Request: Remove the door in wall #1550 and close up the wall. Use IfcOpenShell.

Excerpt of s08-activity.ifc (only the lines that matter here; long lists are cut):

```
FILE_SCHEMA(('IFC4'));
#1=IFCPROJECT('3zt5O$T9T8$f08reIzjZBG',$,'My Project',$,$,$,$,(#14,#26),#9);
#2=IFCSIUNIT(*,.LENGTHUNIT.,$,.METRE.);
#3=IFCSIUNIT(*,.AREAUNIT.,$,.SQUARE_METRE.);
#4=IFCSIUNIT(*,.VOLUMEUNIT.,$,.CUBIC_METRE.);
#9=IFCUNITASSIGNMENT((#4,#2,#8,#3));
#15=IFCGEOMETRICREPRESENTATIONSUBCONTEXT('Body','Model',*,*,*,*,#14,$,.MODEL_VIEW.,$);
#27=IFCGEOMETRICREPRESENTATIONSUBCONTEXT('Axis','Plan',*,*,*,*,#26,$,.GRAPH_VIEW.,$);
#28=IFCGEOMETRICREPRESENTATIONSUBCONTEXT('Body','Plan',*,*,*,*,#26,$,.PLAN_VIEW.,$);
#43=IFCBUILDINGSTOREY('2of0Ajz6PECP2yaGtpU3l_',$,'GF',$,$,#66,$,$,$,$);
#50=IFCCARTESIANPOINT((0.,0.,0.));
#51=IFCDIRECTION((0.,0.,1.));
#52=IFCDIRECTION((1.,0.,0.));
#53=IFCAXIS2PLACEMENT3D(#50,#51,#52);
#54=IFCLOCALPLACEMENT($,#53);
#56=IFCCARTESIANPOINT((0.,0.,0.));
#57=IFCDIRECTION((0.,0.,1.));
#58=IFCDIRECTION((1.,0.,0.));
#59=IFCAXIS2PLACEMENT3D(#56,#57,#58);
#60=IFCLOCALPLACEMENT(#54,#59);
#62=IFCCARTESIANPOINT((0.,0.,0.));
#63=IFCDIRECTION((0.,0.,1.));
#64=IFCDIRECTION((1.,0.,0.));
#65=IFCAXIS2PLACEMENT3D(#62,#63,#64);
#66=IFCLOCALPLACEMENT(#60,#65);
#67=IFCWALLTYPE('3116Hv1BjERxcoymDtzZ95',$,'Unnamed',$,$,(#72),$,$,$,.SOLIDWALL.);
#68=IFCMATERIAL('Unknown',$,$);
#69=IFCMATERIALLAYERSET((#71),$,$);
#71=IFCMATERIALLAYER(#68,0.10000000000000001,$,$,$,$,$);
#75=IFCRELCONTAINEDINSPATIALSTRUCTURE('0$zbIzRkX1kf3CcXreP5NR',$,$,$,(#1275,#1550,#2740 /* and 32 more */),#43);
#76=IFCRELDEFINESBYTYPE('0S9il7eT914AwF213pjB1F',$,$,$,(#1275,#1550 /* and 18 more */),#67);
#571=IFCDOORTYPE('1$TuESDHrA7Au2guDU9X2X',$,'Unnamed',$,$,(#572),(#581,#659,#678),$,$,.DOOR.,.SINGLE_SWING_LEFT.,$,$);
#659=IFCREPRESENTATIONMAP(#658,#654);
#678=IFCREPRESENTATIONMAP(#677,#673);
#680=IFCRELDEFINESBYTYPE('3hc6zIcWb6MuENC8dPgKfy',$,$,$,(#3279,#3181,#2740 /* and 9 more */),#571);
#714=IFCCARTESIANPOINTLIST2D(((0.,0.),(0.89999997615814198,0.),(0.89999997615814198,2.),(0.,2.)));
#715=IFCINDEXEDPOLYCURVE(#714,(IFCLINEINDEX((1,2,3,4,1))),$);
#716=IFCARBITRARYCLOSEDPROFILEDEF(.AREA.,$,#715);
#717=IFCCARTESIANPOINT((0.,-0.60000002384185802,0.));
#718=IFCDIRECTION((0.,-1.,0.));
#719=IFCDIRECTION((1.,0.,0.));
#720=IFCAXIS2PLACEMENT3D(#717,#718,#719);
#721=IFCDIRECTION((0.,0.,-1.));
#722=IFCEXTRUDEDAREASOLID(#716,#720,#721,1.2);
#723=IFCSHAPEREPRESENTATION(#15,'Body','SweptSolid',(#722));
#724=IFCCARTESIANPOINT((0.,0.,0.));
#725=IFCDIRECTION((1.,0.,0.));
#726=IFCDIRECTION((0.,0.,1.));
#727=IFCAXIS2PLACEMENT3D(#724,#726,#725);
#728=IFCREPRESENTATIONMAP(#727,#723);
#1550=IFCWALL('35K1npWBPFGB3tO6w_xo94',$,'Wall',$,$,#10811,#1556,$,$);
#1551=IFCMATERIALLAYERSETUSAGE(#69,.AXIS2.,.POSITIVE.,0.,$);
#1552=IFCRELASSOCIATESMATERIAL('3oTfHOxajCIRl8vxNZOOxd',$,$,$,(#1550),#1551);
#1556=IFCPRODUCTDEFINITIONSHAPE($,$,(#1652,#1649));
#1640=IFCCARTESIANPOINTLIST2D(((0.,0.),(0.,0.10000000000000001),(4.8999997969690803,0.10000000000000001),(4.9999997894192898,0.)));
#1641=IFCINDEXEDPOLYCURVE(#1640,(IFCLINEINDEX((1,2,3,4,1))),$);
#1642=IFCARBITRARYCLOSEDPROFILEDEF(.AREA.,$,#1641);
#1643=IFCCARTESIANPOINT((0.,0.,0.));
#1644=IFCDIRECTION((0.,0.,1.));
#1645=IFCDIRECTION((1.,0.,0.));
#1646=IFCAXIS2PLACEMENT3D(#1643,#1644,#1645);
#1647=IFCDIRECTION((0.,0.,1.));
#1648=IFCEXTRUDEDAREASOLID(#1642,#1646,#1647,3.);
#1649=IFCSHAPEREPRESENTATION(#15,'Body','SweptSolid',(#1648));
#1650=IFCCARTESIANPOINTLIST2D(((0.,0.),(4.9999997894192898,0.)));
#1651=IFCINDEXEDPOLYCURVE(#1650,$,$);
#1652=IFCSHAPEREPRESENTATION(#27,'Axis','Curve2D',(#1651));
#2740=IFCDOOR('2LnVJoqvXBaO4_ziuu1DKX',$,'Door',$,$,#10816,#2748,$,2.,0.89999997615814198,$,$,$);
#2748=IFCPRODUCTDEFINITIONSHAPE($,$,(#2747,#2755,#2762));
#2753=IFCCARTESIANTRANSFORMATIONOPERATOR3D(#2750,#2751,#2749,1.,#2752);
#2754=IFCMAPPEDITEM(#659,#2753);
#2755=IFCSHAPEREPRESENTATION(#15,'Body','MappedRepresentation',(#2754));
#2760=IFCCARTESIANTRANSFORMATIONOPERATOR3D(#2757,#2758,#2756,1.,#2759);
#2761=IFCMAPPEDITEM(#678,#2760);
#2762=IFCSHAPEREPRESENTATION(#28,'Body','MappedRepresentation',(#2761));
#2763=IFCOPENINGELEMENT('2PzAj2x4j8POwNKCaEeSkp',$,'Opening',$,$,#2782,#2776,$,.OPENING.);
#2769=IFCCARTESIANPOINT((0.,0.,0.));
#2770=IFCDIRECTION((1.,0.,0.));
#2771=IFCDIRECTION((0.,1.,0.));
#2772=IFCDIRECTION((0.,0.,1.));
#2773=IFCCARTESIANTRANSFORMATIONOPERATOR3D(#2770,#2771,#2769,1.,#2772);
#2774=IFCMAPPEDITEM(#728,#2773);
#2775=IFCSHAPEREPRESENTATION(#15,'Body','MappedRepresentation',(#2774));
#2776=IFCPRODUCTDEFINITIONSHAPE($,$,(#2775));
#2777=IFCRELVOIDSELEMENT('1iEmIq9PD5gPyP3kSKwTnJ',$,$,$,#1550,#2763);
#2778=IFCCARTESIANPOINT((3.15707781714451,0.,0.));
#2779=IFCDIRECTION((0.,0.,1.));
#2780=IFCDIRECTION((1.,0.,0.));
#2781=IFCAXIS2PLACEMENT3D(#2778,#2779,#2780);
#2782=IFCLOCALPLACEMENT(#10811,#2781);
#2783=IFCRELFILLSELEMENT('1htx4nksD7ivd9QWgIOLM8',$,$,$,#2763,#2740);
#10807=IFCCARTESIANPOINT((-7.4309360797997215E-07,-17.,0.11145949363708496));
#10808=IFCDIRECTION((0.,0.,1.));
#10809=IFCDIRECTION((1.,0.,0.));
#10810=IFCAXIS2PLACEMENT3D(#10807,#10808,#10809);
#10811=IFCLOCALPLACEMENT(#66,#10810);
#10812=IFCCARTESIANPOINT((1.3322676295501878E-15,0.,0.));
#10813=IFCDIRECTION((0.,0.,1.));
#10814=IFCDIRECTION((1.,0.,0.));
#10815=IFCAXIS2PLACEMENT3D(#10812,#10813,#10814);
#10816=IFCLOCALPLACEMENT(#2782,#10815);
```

```python
import ifcopenshell
import ifcopenshell.api.feature
import ifcopenshell.api.root
import ifcopenshell.geom
import ifcopenshell.util.shape

model = ifcopenshell.open("s08-activity.ifc")
settings = ifcopenshell.geom.settings()


def volume(element):
    """Net volume in cubic metres, openings subtracted."""
    shape = ifcopenshell.geom.create_shape(settings, element)
    return ifcopenshell.util.shape.get_volume(shape.geometry)


door = model.by_guid("2LnVJoqvXBaO4_ziuu1DKX")
opening = door.FillsVoids[0].RelatingOpeningElement
wall = opening.VoidsElements[0].RelatingBuildingElement
before = volume(wall)

ifcopenshell.api.root.remove_product(model, product=door)
ifcopenshell.api.feature.remove_feature(model, feature=opening)

after = volume(wall)

print(f"wall volume {before:.3f} -> {after:.3f} m3")

model.write("s08-activity-out.ifc")
```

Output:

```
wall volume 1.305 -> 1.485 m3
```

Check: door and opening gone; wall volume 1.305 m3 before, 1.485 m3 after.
